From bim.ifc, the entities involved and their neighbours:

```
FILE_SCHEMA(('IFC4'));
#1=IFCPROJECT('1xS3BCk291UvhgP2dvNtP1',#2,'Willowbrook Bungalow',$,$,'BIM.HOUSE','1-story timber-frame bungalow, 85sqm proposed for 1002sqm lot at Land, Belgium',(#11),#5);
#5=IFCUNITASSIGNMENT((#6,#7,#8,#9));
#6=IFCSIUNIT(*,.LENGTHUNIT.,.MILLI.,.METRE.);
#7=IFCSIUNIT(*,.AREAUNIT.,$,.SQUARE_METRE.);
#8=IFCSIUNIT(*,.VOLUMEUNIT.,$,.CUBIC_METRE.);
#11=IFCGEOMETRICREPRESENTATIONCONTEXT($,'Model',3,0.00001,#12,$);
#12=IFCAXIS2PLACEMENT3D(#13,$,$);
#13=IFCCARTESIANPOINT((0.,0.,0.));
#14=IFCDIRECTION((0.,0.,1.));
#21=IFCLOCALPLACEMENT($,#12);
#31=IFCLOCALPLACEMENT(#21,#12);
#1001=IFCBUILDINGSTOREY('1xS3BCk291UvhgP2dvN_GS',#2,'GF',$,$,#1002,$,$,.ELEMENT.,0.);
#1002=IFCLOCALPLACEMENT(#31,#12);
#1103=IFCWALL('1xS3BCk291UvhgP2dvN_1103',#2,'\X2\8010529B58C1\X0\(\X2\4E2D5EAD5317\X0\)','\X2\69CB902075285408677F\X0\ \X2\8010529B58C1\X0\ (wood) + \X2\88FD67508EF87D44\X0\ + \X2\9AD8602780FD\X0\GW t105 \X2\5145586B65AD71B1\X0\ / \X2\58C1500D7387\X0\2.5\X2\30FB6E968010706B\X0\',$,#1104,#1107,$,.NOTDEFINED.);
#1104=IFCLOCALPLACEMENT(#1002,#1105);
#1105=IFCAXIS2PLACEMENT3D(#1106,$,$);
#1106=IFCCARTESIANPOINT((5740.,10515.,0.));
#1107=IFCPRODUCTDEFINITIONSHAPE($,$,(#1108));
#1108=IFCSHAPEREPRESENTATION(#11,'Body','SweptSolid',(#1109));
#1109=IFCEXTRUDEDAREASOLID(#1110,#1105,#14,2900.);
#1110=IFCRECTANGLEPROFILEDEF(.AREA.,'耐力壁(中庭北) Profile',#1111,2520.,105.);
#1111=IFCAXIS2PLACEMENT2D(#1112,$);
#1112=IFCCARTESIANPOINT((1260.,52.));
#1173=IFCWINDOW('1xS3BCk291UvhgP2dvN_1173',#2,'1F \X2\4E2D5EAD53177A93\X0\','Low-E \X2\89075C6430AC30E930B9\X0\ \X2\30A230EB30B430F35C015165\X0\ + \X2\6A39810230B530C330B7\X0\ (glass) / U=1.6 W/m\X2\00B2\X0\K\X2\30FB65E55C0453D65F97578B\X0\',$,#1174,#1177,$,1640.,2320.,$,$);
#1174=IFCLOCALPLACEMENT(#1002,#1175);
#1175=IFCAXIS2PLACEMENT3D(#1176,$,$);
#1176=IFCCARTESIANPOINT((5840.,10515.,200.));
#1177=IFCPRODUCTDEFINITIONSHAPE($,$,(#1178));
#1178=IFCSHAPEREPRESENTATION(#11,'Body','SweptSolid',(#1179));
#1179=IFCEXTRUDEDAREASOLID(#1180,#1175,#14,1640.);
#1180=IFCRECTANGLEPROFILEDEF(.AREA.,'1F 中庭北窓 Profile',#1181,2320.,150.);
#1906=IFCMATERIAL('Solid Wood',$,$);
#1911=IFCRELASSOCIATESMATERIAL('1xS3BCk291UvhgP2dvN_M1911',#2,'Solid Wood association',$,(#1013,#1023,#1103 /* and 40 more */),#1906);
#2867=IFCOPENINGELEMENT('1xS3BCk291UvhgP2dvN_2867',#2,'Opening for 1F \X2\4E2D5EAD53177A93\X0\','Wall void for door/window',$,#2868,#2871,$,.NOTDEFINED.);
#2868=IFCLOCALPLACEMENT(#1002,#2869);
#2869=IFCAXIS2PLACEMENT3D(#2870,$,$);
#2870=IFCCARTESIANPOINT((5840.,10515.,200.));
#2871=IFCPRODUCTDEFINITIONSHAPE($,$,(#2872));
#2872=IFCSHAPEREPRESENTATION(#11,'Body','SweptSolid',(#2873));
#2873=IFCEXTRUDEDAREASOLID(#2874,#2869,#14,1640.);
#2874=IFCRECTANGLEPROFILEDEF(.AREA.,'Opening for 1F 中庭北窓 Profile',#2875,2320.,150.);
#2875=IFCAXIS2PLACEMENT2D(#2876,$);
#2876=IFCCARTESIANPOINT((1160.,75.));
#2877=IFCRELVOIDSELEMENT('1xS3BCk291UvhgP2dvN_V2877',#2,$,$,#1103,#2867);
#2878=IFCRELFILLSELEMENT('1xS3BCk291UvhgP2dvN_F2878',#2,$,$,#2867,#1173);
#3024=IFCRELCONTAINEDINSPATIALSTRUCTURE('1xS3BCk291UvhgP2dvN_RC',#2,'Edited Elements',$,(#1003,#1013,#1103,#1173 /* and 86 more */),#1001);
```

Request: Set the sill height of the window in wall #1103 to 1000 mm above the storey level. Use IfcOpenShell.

```python
import numpy as np
import ifcopenshell
import ifcopenshell.api.geometry
import ifcopenshell.geom
import ifcopenshell.util.element
import ifcopenshell.util.placement
import ifcopenshell.util.shape
import ifcopenshell.util.unit

model = ifcopenshell.open("bim.ifc")
unit_scale = ifcopenshell.util.unit.calculate_unit_scale(model)

window = model.by_guid("1xS3BCk291UvhgP2dvN_1173")
opening = window.FillsVoids[0].RelatingOpeningElement
storey = ifcopenshell.util.element.get_container(window, ifc_class="IfcBuildingStorey")
level = ifcopenshell.util.placement.get_local_placement(storey.ObjectPlacement)[2, 3]

# The opening's origin need not be at the sill, so measure its lowest point.
shape = ifcopenshell.geom.create_shape(ifcopenshell.geom.settings(), opening)
bottom = ifcopenshell.util.shape.get_shape_bottom_elevation(shape, shape.geometry) / unit_scale
dz = level + 1000.0 - bottom

shift = np.array([0.0, 0.0, dz])
# The window is not placed relative to its opening, so move both.
for product in (opening, window):
    matrix = ifcopenshell.util.placement.get_local_placement(product.ObjectPlacement)
    matrix[:3, 3] += shift
    ifcopenshell.api.geometry.edit_object_placement(model, product=product, matrix=matrix, is_si=False)

print(f"moved by {dz * unit_scale:+.3f} m")

model.write("bim_rev.ifc")
```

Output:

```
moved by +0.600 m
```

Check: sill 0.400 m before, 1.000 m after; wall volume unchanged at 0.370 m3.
